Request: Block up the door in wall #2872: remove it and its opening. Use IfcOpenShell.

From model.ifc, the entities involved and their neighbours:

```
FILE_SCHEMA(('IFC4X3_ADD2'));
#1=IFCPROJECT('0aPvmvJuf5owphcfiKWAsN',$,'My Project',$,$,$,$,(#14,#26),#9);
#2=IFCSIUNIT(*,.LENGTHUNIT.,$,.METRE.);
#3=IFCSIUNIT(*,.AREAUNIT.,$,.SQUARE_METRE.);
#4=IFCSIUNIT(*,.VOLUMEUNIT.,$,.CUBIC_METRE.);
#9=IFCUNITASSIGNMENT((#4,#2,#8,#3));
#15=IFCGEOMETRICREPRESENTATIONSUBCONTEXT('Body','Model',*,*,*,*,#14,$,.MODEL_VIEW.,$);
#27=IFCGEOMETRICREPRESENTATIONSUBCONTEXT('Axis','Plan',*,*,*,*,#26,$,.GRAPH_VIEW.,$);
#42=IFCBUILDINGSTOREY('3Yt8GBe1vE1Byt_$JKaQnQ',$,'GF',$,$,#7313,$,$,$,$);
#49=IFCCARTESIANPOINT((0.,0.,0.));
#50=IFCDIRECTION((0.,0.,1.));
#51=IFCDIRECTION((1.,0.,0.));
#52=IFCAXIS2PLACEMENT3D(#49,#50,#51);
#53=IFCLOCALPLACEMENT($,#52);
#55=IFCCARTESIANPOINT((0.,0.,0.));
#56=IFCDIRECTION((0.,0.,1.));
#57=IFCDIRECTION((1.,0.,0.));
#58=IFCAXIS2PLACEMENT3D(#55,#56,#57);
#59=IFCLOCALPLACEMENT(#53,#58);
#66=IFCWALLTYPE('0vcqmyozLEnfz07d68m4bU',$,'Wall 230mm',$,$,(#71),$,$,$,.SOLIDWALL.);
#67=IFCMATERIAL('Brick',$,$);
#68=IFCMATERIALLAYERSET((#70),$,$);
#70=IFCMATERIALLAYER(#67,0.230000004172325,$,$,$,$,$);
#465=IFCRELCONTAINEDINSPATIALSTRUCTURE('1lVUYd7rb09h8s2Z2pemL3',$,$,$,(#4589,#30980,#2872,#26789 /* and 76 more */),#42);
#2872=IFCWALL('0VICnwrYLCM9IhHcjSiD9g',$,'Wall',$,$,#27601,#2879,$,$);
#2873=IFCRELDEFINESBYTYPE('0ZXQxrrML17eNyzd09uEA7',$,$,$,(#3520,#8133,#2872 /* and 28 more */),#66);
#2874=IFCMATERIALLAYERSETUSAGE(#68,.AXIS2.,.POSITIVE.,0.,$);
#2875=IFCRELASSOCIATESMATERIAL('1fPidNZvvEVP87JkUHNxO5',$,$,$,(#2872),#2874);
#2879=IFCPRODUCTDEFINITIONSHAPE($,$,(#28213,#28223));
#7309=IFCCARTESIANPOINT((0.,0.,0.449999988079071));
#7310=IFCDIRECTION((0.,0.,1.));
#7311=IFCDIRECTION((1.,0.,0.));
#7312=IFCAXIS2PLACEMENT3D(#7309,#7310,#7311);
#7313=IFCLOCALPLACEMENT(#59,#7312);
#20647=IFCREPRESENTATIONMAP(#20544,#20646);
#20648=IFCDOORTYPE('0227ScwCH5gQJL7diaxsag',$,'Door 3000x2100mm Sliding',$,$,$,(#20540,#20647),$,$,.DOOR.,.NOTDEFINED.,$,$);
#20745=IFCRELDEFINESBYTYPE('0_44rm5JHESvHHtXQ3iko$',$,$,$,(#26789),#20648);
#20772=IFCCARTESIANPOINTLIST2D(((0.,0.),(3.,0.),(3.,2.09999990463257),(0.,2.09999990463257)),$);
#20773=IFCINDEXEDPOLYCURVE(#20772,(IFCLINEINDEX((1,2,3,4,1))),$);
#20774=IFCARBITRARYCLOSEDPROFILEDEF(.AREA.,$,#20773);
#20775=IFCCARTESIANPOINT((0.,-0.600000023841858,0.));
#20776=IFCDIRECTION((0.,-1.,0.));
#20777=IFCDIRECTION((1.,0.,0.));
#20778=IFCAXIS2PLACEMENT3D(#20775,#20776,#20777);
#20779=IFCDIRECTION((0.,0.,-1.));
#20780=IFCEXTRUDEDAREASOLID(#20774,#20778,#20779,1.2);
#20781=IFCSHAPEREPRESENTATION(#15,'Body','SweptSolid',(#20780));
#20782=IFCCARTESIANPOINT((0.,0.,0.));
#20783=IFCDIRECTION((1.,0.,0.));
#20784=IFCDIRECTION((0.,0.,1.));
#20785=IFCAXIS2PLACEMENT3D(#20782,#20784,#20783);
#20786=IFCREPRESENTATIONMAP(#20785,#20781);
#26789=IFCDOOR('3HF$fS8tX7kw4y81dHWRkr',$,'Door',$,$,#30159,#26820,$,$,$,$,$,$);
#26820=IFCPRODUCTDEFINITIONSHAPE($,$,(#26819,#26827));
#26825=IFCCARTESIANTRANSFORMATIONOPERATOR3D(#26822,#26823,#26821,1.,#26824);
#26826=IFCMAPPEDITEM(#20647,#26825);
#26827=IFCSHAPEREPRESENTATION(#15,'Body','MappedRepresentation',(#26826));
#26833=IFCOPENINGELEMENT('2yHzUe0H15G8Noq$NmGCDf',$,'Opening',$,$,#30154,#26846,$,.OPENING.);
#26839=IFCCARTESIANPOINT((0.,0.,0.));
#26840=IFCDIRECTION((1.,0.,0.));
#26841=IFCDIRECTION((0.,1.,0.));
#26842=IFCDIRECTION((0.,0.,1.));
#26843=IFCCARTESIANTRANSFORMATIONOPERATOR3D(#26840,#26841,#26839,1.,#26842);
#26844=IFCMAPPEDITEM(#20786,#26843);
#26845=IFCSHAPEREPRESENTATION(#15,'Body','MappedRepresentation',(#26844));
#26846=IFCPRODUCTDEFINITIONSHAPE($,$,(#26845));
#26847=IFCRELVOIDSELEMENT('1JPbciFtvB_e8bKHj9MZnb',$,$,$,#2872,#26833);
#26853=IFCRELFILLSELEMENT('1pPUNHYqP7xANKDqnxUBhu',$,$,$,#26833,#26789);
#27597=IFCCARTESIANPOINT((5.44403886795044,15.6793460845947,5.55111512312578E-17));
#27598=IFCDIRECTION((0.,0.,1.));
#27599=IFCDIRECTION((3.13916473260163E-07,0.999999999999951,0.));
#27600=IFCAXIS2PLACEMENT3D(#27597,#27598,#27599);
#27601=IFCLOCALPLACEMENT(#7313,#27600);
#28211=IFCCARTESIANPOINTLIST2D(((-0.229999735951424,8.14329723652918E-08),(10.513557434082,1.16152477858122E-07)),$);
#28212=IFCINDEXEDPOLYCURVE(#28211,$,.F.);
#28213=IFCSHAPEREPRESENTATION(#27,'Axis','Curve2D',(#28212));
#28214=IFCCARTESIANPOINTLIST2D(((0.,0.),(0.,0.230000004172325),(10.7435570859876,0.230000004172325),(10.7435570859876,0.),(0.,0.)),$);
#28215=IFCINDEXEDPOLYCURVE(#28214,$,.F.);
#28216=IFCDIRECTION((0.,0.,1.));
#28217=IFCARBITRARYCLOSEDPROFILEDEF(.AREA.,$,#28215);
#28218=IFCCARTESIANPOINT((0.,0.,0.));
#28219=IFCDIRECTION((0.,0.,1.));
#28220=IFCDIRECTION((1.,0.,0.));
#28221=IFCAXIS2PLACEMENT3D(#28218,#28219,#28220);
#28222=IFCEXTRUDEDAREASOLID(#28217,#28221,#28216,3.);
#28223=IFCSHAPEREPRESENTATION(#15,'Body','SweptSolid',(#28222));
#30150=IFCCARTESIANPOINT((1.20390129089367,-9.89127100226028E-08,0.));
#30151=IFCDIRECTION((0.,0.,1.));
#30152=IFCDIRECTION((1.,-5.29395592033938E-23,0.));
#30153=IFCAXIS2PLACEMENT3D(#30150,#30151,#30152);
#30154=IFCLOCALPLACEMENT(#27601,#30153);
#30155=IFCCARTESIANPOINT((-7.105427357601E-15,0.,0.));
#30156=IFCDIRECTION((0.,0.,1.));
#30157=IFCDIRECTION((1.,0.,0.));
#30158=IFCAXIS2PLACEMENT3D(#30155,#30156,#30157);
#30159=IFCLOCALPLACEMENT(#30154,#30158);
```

```python
import ifcopenshell
import ifcopenshell.api.feature
import ifcopenshell.api.root
import ifcopenshell.geom
import ifcopenshell.util.shape

model = ifcopenshell.open("model.ifc")
settings = ifcopenshell.geom.settings()


def volume(element):
    """Net volume in cubic metres, openings subtracted."""
    shape = ifcopenshell.geom.create_shape(settings, element)
    return ifcopenshell.util.shape.get_volume(shape.geometry)


door = model.by_guid("3HF$fS8tX7kw4y81dHWRkr")
opening = door.FillsVoids[0].RelatingOpeningElement
wall = opening.VoidsElements[0].RelatingBuildingElement
before = volume(wall)

ifcopenshell.api.root.remove_product(model, product=door)
ifcopenshell.api.feature.remove_feature(model, feature=opening)

after = volume(wall)

print(f"wall volume {before:.3f} -> {after:.3f} m3")

model.write("model_v2.ifc")
```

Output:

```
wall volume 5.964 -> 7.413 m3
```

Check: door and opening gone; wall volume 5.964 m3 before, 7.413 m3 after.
